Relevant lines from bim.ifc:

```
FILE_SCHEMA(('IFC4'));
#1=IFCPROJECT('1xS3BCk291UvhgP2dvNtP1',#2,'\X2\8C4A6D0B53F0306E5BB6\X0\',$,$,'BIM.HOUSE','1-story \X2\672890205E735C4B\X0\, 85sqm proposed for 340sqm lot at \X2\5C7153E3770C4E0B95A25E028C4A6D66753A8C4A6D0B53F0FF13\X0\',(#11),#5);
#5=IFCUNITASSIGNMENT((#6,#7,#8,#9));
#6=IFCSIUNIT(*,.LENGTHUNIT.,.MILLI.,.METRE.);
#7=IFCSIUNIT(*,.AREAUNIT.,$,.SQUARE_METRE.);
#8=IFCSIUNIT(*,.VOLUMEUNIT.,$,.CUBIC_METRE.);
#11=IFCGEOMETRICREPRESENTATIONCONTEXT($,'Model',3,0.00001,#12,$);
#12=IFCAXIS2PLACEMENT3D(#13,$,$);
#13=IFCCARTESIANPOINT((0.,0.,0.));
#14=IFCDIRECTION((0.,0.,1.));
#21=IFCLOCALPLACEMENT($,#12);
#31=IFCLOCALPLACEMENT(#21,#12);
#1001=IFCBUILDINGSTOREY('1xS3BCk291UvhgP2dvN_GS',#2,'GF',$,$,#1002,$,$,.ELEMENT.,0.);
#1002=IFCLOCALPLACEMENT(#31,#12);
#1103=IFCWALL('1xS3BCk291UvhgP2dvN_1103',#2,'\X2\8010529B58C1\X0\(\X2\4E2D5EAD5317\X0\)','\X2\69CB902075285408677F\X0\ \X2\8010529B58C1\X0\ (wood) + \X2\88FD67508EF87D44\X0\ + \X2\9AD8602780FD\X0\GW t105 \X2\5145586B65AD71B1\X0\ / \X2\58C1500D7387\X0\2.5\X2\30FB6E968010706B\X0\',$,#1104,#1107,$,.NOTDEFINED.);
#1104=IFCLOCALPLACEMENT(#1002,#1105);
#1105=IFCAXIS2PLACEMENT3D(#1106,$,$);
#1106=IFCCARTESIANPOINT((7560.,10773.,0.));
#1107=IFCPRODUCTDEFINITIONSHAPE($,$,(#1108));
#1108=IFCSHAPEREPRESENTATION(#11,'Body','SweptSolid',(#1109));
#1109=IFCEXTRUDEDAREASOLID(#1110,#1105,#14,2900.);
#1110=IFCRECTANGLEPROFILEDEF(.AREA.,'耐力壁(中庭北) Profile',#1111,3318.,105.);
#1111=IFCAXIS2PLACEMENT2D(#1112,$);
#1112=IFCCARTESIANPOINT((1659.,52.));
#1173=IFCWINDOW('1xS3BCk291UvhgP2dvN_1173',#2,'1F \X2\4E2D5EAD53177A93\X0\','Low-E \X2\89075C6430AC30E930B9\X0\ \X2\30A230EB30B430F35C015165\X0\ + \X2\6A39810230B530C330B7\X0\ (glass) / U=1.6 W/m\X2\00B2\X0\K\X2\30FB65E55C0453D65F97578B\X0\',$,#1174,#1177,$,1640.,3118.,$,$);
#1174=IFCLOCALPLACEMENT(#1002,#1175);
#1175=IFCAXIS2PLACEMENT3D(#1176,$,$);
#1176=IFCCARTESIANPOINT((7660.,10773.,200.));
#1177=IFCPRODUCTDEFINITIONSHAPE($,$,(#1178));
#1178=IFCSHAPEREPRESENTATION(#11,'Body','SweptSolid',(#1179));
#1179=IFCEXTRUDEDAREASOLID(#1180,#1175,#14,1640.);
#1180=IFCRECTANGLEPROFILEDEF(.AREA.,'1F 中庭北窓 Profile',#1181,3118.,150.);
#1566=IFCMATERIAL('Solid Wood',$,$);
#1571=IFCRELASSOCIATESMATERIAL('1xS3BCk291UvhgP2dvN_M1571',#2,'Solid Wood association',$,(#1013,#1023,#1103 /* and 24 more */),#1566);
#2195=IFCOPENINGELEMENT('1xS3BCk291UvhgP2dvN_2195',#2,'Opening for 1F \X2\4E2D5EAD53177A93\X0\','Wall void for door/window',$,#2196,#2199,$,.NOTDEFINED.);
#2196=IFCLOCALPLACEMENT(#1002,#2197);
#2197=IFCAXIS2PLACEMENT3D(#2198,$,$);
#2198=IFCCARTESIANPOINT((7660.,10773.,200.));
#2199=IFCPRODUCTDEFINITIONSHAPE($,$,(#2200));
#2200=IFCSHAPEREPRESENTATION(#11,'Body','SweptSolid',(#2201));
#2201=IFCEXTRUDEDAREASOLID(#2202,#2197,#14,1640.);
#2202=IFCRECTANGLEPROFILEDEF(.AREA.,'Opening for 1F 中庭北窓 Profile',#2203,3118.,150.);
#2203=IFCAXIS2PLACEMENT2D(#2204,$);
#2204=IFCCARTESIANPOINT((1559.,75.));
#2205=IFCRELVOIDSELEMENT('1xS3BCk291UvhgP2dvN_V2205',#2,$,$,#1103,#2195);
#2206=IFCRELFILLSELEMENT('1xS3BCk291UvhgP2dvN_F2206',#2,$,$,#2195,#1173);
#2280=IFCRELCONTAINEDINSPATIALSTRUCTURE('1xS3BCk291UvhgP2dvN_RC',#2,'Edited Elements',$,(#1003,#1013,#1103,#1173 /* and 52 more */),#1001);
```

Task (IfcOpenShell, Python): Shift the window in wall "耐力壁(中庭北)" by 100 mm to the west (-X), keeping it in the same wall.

```python
import ifcopenshell
import ifcopenshell.api.geometry
import ifcopenshell.util.placement
import ifcopenshell.util.unit

model = ifcopenshell.open("bim.ifc")
unit_scale = ifcopenshell.util.unit.calculate_unit_scale(model)

window = model.by_guid("1xS3BCk291UvhgP2dvN_1173")
opening = window.FillsVoids[0].RelatingOpeningElement
wall = opening.VoidsElements[0].RelatingBuildingElement

wall_matrix = ifcopenshell.util.placement.get_local_placement(wall.ObjectPlacement)
shift = wall_matrix[:3, 0] * -0.1 / unit_scale
before = ifcopenshell.util.placement.get_local_placement(window.ObjectPlacement)[:3, 3].copy()

# The window is not placed relative to its opening, so move both.
for product in (opening, window):
    matrix = ifcopenshell.util.placement.get_local_placement(product.ObjectPlacement)
    matrix[:3, 3] += shift
    ifcopenshell.api.geometry.edit_object_placement(model, product=product, matrix=matrix, is_si=False)

after = ifcopenshell.util.placement.get_local_placement(window.ObjectPlacement)[:3, 3]
print("window moved by", (after - before).round(3) + 0.0)

model.write("bim_edited.ifc")
```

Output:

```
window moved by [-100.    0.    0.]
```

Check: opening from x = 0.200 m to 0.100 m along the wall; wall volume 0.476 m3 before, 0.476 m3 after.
